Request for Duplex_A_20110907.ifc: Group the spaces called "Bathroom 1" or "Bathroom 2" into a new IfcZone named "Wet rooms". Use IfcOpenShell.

First a look at what the model holds.

```python
import ifcopenshell

model = ifcopenshell.open("Duplex_A_20110907.ifc")
print(model.schema)
seen = {}
for space in model.by_type("IfcSpace"):
    seen[space.LongName] = seen.get(space.LongName, 0) + 1
for name, count in sorted(seen.items(), key=str):
    print(count, "x", name)
print("zones:", [z.Name for z in model.by_type("IfcZone")][:20])
```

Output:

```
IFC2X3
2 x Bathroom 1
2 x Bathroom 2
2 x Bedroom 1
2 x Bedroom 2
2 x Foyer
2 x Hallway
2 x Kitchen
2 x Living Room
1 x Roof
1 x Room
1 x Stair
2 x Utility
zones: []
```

```python
import ifcopenshell
import ifcopenshell.api.group
import ifcopenshell.api.root

model = ifcopenshell.open("Duplex_A_20110907.ifc")

names = {"Bathroom 1", "Bathroom 2"}
spaces = [s for s in model.by_type("IfcSpace") if s.LongName in names]

zone = ifcopenshell.api.root.create_entity(model, ifc_class="IfcZone", name="Wet rooms")
ifcopenshell.api.group.assign_group(model, products=spaces, group=zone)
print(len(spaces), "spaces in", zone.Name)

model.write("Duplex_A_20110907_updated.ifc")
```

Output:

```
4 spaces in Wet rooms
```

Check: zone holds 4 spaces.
